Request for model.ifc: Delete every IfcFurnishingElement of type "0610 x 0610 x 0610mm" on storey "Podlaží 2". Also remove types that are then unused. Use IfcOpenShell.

First a look at what the model holds.

```python
import ifcopenshell
import ifcopenshell.util.element

model = ifcopenshell.open("model.ifc")
print(model.schema)
storey = next(s for s in model.by_type("IfcBuildingStorey") if s.Name == "Podlaží 2")
furniture = [e for e in ifcopenshell.util.element.get_decomposition(storey) if e.is_a("IfcFurnishingElement")]
seen = {}
for e in furniture:
    element_type = ifcopenshell.util.element.get_type(e)
    name = element_type.Name if element_type not in (None, e) else None
    seen[name] = seen.get(name, 0) + 1
for name, count in sorted(seen.items(), key=str):
    print(count, "x", name)
```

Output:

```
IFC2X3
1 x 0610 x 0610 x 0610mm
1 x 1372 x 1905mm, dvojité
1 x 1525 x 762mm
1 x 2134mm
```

```python
import ifcopenshell
import ifcopenshell.api.root
import ifcopenshell.util.element

model = ifcopenshell.open("model.ifc")

storey = next(s for s in model.by_type("IfcBuildingStorey") if s.Name == "Podlaží 2")
furniture = [e for e in ifcopenshell.util.element.get_decomposition(storey) if e.is_a("IfcFurnishingElement")]
targets = [e for e in furniture if (t := ifcopenshell.util.element.get_type(e)) not in (None, e) and t.Name == "0610 x 0610 x 0610mm"]
types = {ifcopenshell.util.element.get_type(e) for e in targets} - {None, *targets}

for e in targets:
    ifcopenshell.api.root.remove_product(model, product=e)
print(len(targets), "removed")

unused = [t for t in types if not ifcopenshell.util.element.get_types(t)]
for t in unused:
    ifcopenshell.api.root.remove_product(model, product=t)
print(len(unused), "unused types removed")

model.write("model_rev.ifc")
```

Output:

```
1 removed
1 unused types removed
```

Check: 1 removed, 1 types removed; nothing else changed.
